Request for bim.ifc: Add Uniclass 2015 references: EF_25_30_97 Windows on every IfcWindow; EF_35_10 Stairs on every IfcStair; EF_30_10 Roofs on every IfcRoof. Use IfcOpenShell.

First a look at what the model holds.

```python
import ifcopenshell

model = ifcopenshell.open("bim.ifc")
print(model.schema)
print("classifications:", [c.Name for c in model.by_type("IfcClassification")])
for ifc_class in ("IfcDoor", "IfcRoof", "IfcStair", "IfcWall", "IfcWindow"):
    print(ifc_class, len(model.by_type(ifc_class)))
```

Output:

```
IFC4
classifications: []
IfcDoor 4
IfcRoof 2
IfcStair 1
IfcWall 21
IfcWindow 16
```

```python
import ifcopenshell
import ifcopenshell.api.classification

model = ifcopenshell.open("bim.ifc")

system = ifcopenshell.api.classification.add_classification(model, classification="Uniclass 2015")

codes = {
    "IfcWindow": ("EF_25_30_97", "Windows"),
    "IfcStair": ("EF_35_10", "Stairs"),
    "IfcRoof": ("EF_30_10", "Roofs"),
}
for ifc_class, (code, name) in codes.items():
    products = model.by_type(ifc_class)
    ifcopenshell.api.classification.add_reference(
        model, products=products, classification=system, identification=code, name=name
    )
    print(code, len(products))

model.write("bim_v2.ifc")
```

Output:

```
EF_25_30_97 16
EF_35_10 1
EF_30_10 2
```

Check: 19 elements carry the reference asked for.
